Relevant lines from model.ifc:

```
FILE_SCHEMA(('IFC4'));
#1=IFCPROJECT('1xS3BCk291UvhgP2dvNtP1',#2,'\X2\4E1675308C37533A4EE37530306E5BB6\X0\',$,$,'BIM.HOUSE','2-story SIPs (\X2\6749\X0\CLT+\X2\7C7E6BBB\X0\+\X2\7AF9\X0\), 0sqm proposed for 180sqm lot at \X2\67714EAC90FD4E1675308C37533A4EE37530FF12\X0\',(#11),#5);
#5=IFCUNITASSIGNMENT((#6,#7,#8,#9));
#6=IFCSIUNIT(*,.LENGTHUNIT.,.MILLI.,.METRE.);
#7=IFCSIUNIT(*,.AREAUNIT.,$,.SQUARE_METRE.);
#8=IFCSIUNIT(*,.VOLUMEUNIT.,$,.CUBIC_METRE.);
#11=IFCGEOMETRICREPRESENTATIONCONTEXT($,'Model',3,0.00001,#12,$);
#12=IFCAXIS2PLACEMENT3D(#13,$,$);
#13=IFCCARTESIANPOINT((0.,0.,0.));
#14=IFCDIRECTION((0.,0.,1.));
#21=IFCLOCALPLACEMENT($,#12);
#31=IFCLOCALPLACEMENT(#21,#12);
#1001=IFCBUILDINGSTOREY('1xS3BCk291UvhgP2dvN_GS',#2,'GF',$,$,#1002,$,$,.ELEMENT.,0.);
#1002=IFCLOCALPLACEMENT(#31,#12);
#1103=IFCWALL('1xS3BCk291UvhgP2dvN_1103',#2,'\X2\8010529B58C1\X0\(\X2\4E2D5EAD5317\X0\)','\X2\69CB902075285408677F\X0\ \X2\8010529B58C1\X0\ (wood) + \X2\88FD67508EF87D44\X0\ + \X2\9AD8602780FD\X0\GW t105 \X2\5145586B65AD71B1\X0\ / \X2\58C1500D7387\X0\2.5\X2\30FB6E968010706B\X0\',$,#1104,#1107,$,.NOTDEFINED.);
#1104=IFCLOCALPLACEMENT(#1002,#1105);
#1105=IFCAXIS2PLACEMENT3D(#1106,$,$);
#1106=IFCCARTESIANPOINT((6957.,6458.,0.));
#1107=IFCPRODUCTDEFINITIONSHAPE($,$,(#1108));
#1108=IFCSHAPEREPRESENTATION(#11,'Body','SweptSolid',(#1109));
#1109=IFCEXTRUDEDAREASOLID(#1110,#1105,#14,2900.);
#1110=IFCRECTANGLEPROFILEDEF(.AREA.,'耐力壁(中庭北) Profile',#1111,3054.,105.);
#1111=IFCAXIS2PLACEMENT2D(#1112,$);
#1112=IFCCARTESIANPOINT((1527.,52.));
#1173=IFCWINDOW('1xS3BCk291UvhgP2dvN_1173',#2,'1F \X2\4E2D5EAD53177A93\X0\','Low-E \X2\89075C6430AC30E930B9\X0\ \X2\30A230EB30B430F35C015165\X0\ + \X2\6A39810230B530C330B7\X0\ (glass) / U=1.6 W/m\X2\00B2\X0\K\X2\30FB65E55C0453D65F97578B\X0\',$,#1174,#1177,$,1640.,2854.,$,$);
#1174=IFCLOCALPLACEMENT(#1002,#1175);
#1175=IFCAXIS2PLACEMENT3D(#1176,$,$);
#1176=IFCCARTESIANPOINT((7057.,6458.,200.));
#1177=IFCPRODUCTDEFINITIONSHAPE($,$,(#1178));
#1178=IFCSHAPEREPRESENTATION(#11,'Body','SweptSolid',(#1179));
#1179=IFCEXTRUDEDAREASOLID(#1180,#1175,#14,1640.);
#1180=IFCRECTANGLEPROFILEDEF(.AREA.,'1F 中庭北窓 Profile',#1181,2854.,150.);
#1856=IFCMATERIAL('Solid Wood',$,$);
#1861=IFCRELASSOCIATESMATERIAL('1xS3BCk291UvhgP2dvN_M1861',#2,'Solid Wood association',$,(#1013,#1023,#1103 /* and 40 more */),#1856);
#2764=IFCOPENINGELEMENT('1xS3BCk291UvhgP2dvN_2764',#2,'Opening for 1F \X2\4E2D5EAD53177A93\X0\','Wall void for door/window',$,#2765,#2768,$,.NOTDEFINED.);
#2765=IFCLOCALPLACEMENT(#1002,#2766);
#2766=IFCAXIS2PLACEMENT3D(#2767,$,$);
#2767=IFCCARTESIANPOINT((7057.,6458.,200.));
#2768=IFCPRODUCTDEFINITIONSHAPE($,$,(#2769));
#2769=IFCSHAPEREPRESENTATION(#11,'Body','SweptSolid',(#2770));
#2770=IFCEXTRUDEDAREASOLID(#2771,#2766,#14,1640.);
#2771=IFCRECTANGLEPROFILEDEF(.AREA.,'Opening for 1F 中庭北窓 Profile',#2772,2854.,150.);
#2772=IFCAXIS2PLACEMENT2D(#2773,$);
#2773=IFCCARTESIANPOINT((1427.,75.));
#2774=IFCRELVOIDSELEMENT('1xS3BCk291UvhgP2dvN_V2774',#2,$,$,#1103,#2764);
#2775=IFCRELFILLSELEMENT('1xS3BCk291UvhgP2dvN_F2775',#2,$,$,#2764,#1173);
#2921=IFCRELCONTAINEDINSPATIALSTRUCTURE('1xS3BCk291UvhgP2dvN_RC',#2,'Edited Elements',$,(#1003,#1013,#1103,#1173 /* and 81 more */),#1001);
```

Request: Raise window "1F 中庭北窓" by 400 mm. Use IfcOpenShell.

```python
import numpy as np
import ifcopenshell
import ifcopenshell.api.geometry
import ifcopenshell.util.placement
import ifcopenshell.util.unit

model = ifcopenshell.open("model.ifc")
unit_scale = ifcopenshell.util.unit.calculate_unit_scale(model)

window = model.by_guid("1xS3BCk291UvhgP2dvN_1173")
opening = window.FillsVoids[0].RelatingOpeningElement
dz = 0.4 / unit_scale

shift = np.array([0.0, 0.0, dz])
# The window is not placed relative to its opening, so move both.
for product in (opening, window):
    matrix = ifcopenshell.util.placement.get_local_placement(product.ObjectPlacement)
    matrix[:3, 3] += shift
    ifcopenshell.api.geometry.edit_object_placement(model, product=product, matrix=matrix, is_si=False)

print(f"moved by {dz * unit_scale:+.3f} m")

model.write("model-out.ifc")
```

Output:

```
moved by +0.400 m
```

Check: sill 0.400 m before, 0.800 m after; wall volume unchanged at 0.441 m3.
